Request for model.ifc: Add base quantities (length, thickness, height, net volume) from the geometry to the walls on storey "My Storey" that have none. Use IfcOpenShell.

First a look at what the model holds.

```python
import ifcopenshell
import ifcopenshell.util.element
import ifcopenshell.util.unit

model = ifcopenshell.open("model.ifc")
print(model.schema)
for unit_type in ("LENGTHUNIT", "AREAUNIT", "VOLUMEUNIT"):
    print(unit_type, ifcopenshell.util.unit.calculate_unit_scale(model, unit_type))
storey = next(s for s in model.by_type("IfcBuildingStorey") if s.Name == "My Storey")
walls = [e for e in ifcopenshell.util.element.get_decomposition(storey) if e.is_a("IfcWall")]
for e in sorted(walls, key=lambda e: e.id()):
    print(e.id(), e.is_a(), e.Name, list(ifcopenshell.util.element.get_psets(e, qtos_only=True)), sep=" | ")
```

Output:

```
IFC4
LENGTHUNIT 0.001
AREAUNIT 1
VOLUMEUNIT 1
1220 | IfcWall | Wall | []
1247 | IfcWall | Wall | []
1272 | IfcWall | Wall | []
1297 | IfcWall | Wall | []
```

```python
import ifcopenshell
import ifcopenshell.api.pset
import ifcopenshell.geom
import ifcopenshell.util.element
import ifcopenshell.util.shape
import ifcopenshell.util.unit

model = ifcopenshell.open("model.ifc")
unit_scale = ifcopenshell.util.unit.calculate_unit_scale(model)
volume_scale = ifcopenshell.util.unit.calculate_unit_scale(model, "VOLUMEUNIT")
settings = ifcopenshell.geom.settings()

storey = next(s for s in model.by_type("IfcBuildingStorey") if s.Name == "My Storey")
walls = [e for e in ifcopenshell.util.element.get_decomposition(storey) if e.is_a("IfcWall")]

for e in sorted(walls, key=lambda e: e.id()):
    if ifcopenshell.util.element.get_psets(e, qtos_only=True, should_inherit=False):
        continue
    # Geometry comes back in metres, in the element's own axes.
    shape = ifcopenshell.geom.create_shape(settings, e)
    values = {
        "Length": ifcopenshell.util.shape.get_x(shape.geometry) / unit_scale,
        "Width": ifcopenshell.util.shape.get_y(shape.geometry) / unit_scale,
        "Height": ifcopenshell.util.shape.get_z(shape.geometry) / unit_scale,
        "NetVolume": ifcopenshell.util.shape.get_volume(shape.geometry) / volume_scale,
    }
    qto = ifcopenshell.api.pset.add_qto(model, product=e, name="Qto_WallBaseQuantities")
    ifcopenshell.api.pset.edit_qto(model, qto=qto, properties=values)
    print(e.id(), {k: round(v, 3) for k, v in values.items()})

model.write("model-out.ifc")
```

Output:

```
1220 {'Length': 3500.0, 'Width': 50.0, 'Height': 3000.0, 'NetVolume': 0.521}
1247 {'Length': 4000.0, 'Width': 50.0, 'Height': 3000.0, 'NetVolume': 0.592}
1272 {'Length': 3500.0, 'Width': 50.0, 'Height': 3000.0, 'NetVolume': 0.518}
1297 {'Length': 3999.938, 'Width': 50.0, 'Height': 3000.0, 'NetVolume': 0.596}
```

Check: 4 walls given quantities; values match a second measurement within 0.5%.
